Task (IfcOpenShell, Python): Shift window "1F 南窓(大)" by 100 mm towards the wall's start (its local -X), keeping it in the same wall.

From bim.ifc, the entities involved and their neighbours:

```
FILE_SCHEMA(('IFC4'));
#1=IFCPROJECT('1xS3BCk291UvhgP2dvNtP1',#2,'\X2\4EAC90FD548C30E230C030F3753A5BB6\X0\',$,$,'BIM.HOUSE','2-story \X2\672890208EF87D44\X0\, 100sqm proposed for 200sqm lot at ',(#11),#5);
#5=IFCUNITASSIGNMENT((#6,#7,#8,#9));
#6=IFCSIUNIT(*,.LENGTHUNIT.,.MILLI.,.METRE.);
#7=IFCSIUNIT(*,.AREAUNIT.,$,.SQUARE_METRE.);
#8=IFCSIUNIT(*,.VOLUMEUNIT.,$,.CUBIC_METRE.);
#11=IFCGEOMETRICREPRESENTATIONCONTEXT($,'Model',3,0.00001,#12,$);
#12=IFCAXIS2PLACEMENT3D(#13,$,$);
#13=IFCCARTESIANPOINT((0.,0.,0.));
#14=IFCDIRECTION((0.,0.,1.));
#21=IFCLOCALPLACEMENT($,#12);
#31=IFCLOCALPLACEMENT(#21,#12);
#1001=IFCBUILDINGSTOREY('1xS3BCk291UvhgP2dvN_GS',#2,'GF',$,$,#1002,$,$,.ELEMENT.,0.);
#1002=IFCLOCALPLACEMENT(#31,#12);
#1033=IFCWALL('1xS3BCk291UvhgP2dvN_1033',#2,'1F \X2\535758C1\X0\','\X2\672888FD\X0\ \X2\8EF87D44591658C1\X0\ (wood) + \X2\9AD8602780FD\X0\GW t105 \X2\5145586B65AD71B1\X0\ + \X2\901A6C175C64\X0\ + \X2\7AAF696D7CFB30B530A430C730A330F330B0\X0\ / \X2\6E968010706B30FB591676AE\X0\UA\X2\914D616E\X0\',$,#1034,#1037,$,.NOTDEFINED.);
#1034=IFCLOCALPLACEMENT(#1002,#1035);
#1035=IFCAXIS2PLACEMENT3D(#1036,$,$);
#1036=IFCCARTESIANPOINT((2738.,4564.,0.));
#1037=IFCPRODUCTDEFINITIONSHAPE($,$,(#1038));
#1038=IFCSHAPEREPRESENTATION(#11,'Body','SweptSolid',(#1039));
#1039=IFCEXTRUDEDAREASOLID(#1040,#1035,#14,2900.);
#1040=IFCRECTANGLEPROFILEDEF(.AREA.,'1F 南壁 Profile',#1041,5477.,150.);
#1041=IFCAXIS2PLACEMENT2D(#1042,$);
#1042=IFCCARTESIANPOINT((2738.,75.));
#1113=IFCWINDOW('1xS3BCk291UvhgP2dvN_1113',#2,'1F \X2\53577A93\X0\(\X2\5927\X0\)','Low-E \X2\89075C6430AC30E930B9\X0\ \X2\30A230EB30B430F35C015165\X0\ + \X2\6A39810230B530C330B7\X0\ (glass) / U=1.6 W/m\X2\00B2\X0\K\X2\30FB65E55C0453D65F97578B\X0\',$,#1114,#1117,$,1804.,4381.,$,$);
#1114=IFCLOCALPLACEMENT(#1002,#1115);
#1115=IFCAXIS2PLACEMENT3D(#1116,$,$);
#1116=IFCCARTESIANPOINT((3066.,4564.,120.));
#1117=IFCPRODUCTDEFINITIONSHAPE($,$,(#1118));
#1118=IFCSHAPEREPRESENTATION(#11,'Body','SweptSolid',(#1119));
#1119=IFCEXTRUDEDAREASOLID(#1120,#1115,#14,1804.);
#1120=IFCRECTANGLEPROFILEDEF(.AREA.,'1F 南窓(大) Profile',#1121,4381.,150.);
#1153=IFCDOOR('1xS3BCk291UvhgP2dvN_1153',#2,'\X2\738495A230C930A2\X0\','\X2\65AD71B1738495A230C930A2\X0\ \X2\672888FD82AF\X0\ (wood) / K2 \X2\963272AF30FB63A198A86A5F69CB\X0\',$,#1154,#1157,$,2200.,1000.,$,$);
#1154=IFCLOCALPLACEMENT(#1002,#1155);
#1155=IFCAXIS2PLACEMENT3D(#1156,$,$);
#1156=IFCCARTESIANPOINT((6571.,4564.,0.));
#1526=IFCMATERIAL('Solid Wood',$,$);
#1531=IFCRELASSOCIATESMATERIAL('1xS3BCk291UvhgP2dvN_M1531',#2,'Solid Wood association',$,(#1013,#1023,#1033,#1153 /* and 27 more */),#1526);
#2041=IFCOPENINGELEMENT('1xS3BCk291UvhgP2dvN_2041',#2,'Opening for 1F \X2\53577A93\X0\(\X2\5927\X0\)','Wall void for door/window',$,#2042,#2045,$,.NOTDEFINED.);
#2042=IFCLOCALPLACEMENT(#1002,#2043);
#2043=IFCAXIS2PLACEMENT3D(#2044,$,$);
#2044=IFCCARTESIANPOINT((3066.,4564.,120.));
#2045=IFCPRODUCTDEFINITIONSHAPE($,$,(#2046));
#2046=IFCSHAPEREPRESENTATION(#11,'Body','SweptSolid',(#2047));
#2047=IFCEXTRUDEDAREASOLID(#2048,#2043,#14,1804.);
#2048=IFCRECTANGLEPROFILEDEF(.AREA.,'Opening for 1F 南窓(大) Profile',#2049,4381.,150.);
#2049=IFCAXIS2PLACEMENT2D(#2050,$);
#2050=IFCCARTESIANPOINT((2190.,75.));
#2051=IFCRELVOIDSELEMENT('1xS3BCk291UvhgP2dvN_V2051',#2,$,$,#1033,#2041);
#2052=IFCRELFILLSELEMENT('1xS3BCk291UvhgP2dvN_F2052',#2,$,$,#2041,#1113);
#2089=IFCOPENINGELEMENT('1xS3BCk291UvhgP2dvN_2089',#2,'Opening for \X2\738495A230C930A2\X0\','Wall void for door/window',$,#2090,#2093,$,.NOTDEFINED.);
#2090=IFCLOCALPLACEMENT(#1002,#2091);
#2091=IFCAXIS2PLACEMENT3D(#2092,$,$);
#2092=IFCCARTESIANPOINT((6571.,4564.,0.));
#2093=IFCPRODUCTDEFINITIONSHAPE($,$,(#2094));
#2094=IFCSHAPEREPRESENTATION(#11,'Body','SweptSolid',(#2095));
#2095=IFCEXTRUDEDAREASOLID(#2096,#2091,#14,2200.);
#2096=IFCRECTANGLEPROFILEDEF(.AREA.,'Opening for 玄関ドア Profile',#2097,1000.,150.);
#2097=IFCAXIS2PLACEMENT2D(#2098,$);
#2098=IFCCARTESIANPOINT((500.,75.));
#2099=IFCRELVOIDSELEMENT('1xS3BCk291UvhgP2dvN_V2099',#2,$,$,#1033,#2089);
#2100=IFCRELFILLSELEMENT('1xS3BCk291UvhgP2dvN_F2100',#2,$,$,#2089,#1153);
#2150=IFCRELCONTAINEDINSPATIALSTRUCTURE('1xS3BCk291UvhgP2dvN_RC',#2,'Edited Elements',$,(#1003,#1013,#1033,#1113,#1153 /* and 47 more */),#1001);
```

```python
import ifcopenshell
import ifcopenshell.api.geometry
import ifcopenshell.util.placement
import ifcopenshell.util.unit

model = ifcopenshell.open("bim.ifc")
unit_scale = ifcopenshell.util.unit.calculate_unit_scale(model)

window = model.by_id(1113)
opening = window.FillsVoids[0].RelatingOpeningElement
wall = opening.VoidsElements[0].RelatingBuildingElement

wall_matrix = ifcopenshell.util.placement.get_local_placement(wall.ObjectPlacement)
shift = wall_matrix[:3, 0] * -0.1 / unit_scale
before = ifcopenshell.util.placement.get_local_placement(window.ObjectPlacement)[:3, 3].copy()

# The window is not placed relative to its opening, so move both.
for product in (opening, window):
    matrix = ifcopenshell.util.placement.get_local_placement(product.ObjectPlacement)
    matrix[:3, 3] += shift
    ifcopenshell.api.geometry.edit_object_placement(model, product=product, matrix=matrix, is_si=False)

after = ifcopenshell.util.placement.get_local_placement(window.ObjectPlacement)[:3, 3]
print("window moved by", (after - before).round(3) + 0.0)

model.write("bim_rev.ifc")
```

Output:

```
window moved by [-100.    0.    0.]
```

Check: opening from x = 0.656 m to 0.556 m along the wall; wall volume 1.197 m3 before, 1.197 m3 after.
